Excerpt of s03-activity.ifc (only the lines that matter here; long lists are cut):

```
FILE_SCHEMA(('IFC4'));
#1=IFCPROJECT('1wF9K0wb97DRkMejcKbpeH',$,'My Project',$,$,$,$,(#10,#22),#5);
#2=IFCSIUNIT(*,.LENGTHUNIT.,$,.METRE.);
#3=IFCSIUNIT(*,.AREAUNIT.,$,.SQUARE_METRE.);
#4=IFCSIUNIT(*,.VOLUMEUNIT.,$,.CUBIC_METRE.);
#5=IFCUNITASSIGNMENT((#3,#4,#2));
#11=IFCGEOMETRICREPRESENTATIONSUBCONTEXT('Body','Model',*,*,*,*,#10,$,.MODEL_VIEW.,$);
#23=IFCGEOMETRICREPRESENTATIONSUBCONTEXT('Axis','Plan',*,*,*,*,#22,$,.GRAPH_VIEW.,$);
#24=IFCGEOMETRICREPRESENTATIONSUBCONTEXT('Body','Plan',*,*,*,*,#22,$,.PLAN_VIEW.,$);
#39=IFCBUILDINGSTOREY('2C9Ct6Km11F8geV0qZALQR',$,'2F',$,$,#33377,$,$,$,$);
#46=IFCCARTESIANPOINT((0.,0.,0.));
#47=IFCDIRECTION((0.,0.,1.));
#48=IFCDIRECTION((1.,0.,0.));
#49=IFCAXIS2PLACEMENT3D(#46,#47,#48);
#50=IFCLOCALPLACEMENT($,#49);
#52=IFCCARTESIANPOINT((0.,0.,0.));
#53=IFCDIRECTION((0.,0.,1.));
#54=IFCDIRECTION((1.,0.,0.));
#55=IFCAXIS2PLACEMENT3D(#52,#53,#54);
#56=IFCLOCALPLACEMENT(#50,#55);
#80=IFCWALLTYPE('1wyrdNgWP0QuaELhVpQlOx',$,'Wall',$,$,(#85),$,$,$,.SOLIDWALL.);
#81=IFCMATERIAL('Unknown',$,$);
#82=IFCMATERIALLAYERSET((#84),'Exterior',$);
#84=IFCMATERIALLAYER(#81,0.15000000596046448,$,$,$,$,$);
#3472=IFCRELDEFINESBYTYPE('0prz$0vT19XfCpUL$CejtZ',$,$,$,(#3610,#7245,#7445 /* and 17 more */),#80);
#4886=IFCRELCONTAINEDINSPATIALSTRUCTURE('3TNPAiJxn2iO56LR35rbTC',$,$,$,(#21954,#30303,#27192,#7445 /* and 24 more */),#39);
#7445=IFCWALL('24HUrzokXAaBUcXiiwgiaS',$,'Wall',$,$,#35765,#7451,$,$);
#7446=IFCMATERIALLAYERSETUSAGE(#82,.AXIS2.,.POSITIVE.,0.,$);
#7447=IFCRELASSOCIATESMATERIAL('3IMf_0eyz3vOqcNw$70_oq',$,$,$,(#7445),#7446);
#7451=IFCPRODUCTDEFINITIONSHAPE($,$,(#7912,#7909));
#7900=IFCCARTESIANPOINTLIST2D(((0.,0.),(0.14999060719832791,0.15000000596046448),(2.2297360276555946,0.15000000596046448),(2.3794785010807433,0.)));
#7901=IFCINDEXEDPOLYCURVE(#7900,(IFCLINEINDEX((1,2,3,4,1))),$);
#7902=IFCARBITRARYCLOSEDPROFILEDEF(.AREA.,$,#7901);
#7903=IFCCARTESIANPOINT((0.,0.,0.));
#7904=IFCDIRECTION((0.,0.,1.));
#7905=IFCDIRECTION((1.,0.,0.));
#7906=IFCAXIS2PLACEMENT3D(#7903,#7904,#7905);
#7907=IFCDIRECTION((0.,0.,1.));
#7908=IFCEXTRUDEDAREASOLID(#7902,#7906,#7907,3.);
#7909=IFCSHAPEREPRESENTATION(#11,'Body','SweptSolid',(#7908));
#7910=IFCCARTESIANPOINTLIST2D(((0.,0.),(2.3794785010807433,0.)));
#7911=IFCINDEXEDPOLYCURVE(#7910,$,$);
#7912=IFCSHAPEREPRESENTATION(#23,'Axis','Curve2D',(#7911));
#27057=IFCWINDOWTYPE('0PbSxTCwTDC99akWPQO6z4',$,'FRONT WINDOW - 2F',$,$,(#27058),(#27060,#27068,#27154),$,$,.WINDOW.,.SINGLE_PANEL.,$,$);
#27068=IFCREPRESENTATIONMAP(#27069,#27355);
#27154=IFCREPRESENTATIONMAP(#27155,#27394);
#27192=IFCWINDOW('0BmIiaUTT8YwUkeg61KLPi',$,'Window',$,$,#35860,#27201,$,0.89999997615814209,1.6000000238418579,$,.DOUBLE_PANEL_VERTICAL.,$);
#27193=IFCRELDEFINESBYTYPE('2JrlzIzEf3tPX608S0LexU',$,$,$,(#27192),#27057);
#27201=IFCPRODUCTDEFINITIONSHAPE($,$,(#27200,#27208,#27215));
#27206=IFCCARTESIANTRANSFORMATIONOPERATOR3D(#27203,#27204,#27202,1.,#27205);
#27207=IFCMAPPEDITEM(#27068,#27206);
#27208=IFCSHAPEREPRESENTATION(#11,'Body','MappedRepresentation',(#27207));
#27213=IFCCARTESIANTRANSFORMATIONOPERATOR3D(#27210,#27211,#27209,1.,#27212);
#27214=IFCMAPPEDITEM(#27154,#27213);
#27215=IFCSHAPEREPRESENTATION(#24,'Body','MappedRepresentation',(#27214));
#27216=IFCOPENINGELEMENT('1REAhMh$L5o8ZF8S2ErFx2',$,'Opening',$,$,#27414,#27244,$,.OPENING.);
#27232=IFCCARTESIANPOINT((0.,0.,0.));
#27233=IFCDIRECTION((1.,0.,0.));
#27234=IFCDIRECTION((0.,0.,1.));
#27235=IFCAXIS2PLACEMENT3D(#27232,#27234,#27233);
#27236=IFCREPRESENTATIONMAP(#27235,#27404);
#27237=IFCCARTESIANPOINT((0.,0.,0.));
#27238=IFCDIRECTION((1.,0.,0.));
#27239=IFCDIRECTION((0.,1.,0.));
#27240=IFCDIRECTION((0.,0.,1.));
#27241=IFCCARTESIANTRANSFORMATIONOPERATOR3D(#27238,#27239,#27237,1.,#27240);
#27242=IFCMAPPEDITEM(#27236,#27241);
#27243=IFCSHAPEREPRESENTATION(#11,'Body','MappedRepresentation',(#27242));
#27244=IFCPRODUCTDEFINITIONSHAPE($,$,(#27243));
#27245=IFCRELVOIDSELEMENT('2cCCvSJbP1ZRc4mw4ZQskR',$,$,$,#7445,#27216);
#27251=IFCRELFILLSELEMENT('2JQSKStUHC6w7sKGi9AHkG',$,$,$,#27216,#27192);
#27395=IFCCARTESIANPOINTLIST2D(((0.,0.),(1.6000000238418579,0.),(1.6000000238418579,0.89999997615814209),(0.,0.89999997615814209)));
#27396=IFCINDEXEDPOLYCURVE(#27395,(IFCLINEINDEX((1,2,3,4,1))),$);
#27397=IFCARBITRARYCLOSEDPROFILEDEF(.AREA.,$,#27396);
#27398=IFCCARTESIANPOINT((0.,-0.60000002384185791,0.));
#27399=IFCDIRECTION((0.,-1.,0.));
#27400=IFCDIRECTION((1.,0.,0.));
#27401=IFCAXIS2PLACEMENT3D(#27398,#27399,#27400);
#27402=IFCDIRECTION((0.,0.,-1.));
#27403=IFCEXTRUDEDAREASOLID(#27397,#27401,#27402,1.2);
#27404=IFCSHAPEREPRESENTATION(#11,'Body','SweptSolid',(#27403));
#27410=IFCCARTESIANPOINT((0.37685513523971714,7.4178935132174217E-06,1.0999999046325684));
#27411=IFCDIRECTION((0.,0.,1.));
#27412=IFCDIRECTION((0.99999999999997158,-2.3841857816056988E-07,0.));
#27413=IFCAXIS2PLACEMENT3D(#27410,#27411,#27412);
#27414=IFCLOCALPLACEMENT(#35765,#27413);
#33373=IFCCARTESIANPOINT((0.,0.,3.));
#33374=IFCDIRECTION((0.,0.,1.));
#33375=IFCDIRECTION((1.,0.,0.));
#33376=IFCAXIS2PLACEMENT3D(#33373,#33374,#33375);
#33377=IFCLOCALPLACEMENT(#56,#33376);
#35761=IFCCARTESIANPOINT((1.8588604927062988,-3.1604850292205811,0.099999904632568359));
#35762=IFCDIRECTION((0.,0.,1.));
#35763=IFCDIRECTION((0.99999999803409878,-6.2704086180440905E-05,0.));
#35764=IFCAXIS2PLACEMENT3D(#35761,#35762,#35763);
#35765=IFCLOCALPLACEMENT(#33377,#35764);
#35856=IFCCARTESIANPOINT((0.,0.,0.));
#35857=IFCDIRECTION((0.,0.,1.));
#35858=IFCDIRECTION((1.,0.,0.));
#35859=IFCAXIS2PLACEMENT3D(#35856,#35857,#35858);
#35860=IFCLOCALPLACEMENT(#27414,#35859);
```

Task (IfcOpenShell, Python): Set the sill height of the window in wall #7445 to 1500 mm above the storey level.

```python
import numpy as np
import ifcopenshell
import ifcopenshell.api.geometry
import ifcopenshell.geom
import ifcopenshell.util.element
import ifcopenshell.util.placement
import ifcopenshell.util.shape
import ifcopenshell.util.unit

model = ifcopenshell.open("s03-activity.ifc")
unit_scale = ifcopenshell.util.unit.calculate_unit_scale(model)

window = model.by_guid("0BmIiaUTT8YwUkeg61KLPi")
opening = window.FillsVoids[0].RelatingOpeningElement
storey = ifcopenshell.util.element.get_container(window, ifc_class="IfcBuildingStorey")
level = ifcopenshell.util.placement.get_local_placement(storey.ObjectPlacement)[2, 3]

# The opening's origin need not be at the sill, so measure its lowest point.
shape = ifcopenshell.geom.create_shape(ifcopenshell.geom.settings(), opening)
bottom = ifcopenshell.util.shape.get_shape_bottom_elevation(shape, shape.geometry) / unit_scale
dz = level + 1.5 - bottom

shift = np.array([0.0, 0.0, dz])
# The window is placed relative to its opening, so it follows when the opening moves.
matrix = ifcopenshell.util.placement.get_local_placement(opening.ObjectPlacement)
matrix[:3, 3] += shift
ifcopenshell.api.geometry.edit_object_placement(
    model, product=opening, matrix=matrix, is_si=False, should_transform_children=True
)

print(f"moved by {dz * unit_scale:+.3f} m")

model.write("s03-activity_rev.ifc")
```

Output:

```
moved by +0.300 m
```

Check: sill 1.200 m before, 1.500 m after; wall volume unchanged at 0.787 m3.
